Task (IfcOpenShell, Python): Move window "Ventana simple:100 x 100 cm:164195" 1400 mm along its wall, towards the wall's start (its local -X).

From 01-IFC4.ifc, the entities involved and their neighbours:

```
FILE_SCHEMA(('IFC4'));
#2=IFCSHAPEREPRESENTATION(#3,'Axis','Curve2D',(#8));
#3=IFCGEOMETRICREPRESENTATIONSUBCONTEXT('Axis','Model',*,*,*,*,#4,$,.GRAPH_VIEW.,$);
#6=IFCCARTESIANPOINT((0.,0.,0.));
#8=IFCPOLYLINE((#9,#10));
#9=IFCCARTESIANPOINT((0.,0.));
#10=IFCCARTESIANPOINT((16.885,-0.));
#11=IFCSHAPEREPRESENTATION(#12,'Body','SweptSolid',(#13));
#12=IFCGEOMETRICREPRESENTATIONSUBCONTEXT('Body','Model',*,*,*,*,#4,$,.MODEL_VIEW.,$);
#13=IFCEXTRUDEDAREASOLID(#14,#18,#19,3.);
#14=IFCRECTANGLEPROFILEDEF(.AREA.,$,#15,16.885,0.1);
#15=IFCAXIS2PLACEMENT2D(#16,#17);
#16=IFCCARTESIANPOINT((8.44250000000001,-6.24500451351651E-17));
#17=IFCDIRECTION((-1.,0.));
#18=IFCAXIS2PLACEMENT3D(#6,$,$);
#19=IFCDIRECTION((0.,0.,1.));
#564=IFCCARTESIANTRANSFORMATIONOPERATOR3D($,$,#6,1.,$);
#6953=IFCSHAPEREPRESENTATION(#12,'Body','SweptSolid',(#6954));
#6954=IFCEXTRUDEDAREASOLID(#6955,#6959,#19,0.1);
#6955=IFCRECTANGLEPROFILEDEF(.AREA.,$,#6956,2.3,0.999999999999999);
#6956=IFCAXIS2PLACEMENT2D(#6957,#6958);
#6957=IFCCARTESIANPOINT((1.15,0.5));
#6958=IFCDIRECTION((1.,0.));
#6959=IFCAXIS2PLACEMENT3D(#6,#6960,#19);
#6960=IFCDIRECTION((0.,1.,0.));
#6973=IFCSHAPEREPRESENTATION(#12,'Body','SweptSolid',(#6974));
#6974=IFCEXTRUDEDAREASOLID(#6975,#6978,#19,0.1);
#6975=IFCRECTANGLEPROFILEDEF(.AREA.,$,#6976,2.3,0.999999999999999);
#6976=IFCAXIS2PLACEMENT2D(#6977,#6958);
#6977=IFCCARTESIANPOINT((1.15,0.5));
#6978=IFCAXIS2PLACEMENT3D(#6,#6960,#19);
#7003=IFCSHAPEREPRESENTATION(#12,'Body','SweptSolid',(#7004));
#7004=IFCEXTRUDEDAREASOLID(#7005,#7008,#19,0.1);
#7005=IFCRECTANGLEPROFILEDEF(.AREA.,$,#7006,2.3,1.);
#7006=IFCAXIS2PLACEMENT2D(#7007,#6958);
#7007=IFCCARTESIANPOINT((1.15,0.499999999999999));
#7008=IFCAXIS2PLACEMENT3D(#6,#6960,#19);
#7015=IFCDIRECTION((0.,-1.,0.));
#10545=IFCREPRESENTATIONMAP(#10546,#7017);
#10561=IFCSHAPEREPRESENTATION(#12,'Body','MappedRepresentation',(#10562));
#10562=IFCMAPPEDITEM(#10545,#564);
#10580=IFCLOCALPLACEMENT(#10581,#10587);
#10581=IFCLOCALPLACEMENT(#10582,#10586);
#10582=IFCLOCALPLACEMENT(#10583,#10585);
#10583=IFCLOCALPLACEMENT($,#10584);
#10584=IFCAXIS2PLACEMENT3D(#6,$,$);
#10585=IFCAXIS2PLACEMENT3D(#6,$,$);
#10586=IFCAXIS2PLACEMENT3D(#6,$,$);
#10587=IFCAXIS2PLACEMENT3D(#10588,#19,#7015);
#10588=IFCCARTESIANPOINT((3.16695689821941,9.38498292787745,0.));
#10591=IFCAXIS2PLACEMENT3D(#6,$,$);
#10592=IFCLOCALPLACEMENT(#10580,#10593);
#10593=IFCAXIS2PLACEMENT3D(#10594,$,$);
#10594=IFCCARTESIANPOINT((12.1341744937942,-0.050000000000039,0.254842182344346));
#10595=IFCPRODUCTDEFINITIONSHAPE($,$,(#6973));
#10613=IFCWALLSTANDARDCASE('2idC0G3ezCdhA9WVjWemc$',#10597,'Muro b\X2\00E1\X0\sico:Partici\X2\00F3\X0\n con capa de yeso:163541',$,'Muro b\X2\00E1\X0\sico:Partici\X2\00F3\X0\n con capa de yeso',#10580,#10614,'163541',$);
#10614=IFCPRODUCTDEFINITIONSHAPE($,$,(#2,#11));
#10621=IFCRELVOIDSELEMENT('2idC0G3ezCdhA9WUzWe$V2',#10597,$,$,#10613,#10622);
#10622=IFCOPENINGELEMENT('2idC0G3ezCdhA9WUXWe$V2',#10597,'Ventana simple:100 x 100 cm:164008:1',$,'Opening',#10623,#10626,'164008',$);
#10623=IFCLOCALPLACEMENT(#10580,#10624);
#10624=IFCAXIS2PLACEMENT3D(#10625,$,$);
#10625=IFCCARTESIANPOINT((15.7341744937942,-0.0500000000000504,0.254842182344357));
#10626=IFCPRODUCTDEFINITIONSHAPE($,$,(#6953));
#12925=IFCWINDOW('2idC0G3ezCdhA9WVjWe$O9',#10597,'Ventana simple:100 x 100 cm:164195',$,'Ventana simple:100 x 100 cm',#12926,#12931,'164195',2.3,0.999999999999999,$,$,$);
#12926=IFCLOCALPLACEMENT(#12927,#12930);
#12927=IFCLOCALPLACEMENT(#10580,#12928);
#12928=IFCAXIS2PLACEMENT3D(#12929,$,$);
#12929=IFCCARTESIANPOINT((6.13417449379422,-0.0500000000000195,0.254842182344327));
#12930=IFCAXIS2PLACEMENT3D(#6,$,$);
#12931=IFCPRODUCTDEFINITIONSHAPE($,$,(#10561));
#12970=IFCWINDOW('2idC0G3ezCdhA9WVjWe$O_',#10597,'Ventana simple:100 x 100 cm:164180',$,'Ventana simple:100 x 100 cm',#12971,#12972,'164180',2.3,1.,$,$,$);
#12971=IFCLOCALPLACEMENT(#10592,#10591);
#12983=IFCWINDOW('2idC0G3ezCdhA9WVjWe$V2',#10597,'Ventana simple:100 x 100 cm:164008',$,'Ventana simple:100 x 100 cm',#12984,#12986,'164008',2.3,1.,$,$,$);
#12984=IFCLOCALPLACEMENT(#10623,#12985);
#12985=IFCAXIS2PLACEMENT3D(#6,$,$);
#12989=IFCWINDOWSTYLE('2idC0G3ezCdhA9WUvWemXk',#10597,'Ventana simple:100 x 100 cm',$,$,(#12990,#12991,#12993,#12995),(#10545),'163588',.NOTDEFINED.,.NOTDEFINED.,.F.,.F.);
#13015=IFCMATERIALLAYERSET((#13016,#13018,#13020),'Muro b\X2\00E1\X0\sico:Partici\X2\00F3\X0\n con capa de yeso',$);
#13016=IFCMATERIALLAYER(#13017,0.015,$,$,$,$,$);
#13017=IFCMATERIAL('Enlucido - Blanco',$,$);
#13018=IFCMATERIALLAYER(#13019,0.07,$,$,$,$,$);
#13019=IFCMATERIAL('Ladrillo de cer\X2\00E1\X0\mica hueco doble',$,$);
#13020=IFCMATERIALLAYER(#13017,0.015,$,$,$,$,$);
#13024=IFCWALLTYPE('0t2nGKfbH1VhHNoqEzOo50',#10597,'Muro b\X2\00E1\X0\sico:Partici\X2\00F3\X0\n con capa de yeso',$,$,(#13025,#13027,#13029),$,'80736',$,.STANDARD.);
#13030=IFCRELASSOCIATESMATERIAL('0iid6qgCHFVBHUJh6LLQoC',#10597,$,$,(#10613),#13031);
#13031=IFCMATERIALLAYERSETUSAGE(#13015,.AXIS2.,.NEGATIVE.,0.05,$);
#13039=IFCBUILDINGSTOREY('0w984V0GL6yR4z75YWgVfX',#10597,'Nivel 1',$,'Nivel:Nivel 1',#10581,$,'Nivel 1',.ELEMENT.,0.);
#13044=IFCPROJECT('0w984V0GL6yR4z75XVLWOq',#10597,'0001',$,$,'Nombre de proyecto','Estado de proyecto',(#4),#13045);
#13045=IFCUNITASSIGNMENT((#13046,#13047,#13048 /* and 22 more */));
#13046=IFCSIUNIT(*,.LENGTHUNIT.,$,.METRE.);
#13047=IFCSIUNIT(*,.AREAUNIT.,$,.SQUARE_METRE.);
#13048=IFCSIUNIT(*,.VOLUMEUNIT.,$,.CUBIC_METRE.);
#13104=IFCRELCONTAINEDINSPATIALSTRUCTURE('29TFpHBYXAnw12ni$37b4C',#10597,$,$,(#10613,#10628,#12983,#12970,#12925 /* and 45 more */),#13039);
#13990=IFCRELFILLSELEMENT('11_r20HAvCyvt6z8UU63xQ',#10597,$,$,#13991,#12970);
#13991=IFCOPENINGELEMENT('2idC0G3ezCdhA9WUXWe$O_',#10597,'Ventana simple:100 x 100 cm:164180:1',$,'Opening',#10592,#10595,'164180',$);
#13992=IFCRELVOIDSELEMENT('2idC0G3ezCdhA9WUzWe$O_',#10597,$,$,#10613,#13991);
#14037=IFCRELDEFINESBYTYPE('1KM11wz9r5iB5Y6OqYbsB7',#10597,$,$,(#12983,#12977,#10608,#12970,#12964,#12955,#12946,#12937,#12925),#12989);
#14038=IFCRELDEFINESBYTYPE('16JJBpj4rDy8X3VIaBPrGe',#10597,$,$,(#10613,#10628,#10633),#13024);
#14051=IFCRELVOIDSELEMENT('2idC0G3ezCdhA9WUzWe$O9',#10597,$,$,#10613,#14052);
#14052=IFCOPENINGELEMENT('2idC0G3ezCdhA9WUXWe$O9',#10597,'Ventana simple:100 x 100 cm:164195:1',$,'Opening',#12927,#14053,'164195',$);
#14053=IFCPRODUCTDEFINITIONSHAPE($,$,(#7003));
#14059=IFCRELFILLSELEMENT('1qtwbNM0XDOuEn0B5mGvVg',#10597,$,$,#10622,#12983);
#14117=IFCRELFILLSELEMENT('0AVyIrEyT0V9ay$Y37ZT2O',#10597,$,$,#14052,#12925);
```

```python
import ifcopenshell
import ifcopenshell.api.geometry
import ifcopenshell.util.placement
import ifcopenshell.util.unit

model = ifcopenshell.open("01-IFC4.ifc")
unit_scale = ifcopenshell.util.unit.calculate_unit_scale(model)

window = model.by_guid("2idC0G3ezCdhA9WVjWe$O9")
opening = window.FillsVoids[0].RelatingOpeningElement
wall = opening.VoidsElements[0].RelatingBuildingElement

wall_matrix = ifcopenshell.util.placement.get_local_placement(wall.ObjectPlacement)
shift = wall_matrix[:3, 0] * -1.4 / unit_scale
before = ifcopenshell.util.placement.get_local_placement(window.ObjectPlacement)[:3, 3].copy()

# The window is placed relative to its opening, so it follows when the opening moves.
matrix = ifcopenshell.util.placement.get_local_placement(opening.ObjectPlacement)
matrix[:3, 3] += shift
ifcopenshell.api.geometry.edit_object_placement(
    model, product=opening, matrix=matrix, is_si=False, should_transform_children=True
)

after = ifcopenshell.util.placement.get_local_placement(window.ObjectPlacement)[:3, 3]
print("window moved by", (after - before).round(3) + 0.0)

model.write("01-IFC4_v2.ifc")
```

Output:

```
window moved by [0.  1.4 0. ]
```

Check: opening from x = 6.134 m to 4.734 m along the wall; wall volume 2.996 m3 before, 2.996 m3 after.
